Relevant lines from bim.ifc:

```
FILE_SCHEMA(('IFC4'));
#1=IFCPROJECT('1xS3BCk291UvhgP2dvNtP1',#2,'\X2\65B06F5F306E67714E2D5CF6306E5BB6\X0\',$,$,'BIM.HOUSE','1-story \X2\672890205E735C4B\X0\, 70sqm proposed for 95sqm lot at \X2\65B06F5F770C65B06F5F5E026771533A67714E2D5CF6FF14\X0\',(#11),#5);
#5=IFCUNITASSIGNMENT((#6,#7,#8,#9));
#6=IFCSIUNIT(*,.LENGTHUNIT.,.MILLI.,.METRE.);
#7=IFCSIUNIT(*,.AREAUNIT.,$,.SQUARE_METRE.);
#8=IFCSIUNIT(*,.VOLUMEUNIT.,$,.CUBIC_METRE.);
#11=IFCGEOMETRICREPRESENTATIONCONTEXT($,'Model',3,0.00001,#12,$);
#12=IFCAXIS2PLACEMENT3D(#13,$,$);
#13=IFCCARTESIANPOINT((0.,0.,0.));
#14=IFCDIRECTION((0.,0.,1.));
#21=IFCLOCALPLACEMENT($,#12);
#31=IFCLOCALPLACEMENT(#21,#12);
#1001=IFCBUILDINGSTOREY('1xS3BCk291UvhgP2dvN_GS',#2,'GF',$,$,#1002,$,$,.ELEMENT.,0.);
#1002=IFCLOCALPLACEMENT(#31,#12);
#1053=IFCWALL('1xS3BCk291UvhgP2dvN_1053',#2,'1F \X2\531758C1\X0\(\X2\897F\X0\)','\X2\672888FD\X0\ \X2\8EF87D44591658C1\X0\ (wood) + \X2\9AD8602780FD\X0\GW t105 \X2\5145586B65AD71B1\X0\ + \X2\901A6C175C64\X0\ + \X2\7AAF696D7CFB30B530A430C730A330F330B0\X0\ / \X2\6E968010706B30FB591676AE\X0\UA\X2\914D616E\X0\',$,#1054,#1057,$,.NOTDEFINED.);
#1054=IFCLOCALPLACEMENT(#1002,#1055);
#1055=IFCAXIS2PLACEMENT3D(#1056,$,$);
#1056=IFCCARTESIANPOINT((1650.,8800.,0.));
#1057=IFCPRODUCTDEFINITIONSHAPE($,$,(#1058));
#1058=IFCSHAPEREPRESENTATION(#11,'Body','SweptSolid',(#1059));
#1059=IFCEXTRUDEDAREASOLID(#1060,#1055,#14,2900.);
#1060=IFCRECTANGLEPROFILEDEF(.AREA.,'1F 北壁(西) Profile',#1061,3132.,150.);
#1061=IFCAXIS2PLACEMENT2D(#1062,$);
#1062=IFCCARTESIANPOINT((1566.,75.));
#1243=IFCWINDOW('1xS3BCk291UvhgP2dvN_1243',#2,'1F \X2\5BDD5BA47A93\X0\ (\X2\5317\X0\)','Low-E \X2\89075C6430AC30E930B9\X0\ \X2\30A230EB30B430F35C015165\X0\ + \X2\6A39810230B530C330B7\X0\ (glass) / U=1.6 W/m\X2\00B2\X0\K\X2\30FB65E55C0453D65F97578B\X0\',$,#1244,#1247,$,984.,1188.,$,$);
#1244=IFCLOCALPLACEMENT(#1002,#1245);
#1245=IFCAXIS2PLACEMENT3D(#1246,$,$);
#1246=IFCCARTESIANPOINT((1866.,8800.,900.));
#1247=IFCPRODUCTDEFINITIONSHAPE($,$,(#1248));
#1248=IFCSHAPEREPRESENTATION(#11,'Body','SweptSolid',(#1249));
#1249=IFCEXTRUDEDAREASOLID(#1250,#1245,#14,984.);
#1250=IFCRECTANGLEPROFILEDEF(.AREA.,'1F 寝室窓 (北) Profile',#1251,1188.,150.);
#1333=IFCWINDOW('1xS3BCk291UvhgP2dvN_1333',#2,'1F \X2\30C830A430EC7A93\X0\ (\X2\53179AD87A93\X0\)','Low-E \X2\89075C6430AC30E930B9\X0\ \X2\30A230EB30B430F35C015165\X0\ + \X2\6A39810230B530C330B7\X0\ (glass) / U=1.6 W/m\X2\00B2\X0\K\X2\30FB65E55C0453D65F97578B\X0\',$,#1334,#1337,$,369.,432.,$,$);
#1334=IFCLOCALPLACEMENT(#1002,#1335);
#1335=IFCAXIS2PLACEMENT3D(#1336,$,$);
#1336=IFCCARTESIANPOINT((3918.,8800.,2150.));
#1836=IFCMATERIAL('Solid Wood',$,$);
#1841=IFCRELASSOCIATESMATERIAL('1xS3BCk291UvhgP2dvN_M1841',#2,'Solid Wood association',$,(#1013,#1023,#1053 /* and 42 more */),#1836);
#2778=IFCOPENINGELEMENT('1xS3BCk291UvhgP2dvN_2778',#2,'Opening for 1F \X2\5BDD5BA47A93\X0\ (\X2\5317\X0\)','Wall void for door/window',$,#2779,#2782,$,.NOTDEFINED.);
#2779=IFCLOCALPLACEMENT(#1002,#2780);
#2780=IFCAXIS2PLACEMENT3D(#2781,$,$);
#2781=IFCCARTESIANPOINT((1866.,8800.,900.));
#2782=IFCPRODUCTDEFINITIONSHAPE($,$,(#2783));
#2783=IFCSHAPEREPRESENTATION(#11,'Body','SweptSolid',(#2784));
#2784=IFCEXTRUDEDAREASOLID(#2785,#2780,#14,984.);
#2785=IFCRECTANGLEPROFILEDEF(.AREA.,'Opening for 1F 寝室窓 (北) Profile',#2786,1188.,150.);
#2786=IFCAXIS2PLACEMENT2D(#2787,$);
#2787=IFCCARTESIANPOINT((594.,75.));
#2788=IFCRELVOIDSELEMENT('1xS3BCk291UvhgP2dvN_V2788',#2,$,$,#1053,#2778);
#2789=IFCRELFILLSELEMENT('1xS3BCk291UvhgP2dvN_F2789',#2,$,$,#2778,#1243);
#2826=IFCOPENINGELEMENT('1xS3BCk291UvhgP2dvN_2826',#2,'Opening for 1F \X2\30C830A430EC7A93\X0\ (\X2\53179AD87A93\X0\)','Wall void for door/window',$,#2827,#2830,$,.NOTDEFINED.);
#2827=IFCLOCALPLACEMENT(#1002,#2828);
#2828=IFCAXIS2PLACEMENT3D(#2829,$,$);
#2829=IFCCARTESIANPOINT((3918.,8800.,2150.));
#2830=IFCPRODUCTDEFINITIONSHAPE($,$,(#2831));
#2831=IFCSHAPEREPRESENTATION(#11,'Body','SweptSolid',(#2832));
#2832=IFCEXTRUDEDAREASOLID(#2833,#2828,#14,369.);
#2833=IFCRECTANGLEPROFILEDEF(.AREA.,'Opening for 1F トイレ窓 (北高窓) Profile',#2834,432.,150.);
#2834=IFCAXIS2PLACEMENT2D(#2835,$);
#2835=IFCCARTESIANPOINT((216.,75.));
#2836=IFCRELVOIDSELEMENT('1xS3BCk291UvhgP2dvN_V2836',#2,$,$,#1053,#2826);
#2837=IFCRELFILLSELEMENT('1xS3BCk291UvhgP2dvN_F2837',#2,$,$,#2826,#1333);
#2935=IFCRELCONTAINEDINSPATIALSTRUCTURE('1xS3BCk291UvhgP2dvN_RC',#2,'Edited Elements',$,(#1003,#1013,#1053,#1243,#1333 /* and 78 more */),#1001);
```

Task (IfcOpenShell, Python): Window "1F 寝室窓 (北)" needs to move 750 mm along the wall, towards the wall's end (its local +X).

```python
import ifcopenshell
import ifcopenshell.api.geometry
import ifcopenshell.util.placement
import ifcopenshell.util.unit

model = ifcopenshell.open("bim.ifc")
unit_scale = ifcopenshell.util.unit.calculate_unit_scale(model)

window = model.by_guid("1xS3BCk291UvhgP2dvN_1243")
opening = window.FillsVoids[0].RelatingOpeningElement
wall = opening.VoidsElements[0].RelatingBuildingElement

wall_matrix = ifcopenshell.util.placement.get_local_placement(wall.ObjectPlacement)
shift = wall_matrix[:3, 0] * 0.75 / unit_scale
before = ifcopenshell.util.placement.get_local_placement(window.ObjectPlacement)[:3, 3].copy()

# The window is not placed relative to its opening, so move both.
for product in (opening, window):
    matrix = ifcopenshell.util.placement.get_local_placement(product.ObjectPlacement)
    matrix[:3, 3] += shift
    ifcopenshell.api.geometry.edit_object_placement(model, product=product, matrix=matrix, is_si=False)

after = ifcopenshell.util.placement.get_local_placement(window.ObjectPlacement)[:3, 3]
print("window moved by", (after - before).round(3) + 0.0)

model.write("bim_updated.ifc")
```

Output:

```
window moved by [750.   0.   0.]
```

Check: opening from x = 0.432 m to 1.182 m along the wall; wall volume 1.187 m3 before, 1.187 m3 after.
